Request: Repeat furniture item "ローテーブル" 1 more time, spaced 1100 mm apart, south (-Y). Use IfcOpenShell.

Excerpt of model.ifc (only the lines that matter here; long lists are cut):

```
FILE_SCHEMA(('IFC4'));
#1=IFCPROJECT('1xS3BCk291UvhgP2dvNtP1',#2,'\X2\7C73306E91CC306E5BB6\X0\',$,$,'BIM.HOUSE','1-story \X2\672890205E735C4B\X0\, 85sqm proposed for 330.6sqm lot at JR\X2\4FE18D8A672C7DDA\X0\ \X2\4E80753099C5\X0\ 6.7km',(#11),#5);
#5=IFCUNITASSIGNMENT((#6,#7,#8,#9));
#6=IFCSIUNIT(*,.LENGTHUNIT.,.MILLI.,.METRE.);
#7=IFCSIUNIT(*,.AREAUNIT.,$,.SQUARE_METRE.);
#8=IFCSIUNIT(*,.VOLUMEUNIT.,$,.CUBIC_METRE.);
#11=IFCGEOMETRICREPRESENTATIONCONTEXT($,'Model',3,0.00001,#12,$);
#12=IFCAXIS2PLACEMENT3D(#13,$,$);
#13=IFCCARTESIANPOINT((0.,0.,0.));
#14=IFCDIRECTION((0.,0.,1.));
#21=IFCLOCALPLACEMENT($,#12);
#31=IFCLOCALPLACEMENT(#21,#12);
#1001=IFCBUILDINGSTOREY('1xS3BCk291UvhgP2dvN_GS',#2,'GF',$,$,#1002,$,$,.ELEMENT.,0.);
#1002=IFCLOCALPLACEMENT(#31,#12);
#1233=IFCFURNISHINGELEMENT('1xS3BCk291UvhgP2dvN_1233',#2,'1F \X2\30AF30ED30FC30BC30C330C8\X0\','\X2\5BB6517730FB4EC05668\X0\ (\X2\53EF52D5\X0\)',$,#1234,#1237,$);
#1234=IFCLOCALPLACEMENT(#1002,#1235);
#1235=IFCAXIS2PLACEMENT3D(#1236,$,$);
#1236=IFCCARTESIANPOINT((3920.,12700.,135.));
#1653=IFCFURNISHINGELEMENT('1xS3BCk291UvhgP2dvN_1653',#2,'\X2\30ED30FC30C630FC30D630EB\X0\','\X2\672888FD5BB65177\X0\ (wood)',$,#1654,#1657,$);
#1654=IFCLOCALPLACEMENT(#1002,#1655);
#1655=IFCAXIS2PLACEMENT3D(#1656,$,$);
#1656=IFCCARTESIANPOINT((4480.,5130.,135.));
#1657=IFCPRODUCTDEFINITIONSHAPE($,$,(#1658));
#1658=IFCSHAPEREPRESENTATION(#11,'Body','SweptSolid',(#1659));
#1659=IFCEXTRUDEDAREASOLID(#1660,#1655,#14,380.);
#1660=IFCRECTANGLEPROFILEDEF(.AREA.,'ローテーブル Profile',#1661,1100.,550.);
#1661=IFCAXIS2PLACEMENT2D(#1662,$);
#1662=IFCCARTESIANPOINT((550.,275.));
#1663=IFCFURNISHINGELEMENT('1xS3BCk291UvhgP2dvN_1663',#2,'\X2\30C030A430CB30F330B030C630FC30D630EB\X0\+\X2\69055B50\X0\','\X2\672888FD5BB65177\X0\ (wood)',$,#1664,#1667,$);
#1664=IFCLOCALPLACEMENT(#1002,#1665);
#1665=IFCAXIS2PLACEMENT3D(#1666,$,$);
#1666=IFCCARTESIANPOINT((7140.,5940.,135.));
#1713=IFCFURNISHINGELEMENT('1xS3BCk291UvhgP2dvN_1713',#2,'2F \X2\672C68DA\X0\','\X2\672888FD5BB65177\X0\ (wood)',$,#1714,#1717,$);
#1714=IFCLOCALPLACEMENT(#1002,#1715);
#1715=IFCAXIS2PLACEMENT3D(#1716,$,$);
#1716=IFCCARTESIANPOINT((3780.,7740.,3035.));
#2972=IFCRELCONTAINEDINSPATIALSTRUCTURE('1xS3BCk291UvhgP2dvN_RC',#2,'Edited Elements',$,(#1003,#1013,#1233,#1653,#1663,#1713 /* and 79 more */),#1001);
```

```python
import numpy as np
import ifcopenshell
import ifcopenshell.api.geometry
import ifcopenshell.api.root
import ifcopenshell.util.element
import ifcopenshell.util.placement

model = ifcopenshell.open("model.ifc")


def reuse_history(source, copy):
    """copy_class also copies each property set's owner history, people and application; keep the originals."""
    for rel in copy.IsDefinedBy:
        if rel.is_a("IfcRelDefinesByProperties") and (history := rel.RelatingPropertyDefinition.OwnerHistory):
            rel.RelatingPropertyDefinition.OwnerHistory = source.OwnerHistory
            ifcopenshell.util.element.remove_deep2(model, history)


source = model.by_guid("1xS3BCk291UvhgP2dvN_1653")
base = ifcopenshell.util.placement.get_local_placement(source.ObjectPlacement)
step = np.array([0.0, -1.0, 0.0]) * 1100.0

for i in range(1, 2):
    copy = ifcopenshell.api.root.copy_class(model, product=source)
    copy.Representation = ifcopenshell.util.element.copy_deep(
        model, source.Representation, exclude=["IfcGeometricRepresentationContext", "IfcRepresentationMap"]
    )
    reuse_history(source, copy)
    matrix = base.copy()
    matrix[:3, 3] += i * step
    print("added at", matrix[:3, 3].round(3) + 0.0)
    ifcopenshell.api.geometry.edit_object_placement(model, product=copy, matrix=matrix, is_si=False)

model.write("model_updated.ifc")
```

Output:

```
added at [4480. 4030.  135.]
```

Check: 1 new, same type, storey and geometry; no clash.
